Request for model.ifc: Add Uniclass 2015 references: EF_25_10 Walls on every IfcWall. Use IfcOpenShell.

First a look at what the model holds.

```python
import ifcopenshell

model = ifcopenshell.open("model.ifc")
print(model.schema)
print("classifications:", [c.Name for c in model.by_type("IfcClassification")])
for ifc_class in ("IfcDoor", "IfcRoof", "IfcStair", "IfcWall", "IfcWindow"):
    print(ifc_class, len(model.by_type(ifc_class)))
```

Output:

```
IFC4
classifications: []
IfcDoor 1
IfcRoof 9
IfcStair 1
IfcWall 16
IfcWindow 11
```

```python
import ifcopenshell
import ifcopenshell.api.classification

model = ifcopenshell.open("model.ifc")

system = ifcopenshell.api.classification.add_classification(model, classification="Uniclass 2015")

codes = {
    "IfcWall": ("EF_25_10", "Walls"),
}
for ifc_class, (code, name) in codes.items():
    products = model.by_type(ifc_class)
    ifcopenshell.api.classification.add_reference(
        model, products=products, classification=system, identification=code, name=name
    )
    print(code, len(products))

model.write("model_updated.ifc")
```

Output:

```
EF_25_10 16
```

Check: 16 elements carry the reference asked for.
